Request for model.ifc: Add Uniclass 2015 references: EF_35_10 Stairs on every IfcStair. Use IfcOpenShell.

First a look at what the model holds.

```python
import ifcopenshell

model = ifcopenshell.open("model.ifc")
print(model.schema)
print("classifications:", [c.Name for c in model.by_type("IfcClassification")])
for ifc_class in ("IfcDoor", "IfcRoof", "IfcStair", "IfcWall", "IfcWindow"):
    print(ifc_class, len(model.by_type(ifc_class)))
```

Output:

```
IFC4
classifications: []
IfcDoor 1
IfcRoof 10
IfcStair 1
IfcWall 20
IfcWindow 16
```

```python
import ifcopenshell
import ifcopenshell.api.classification

model = ifcopenshell.open("model.ifc")

system = ifcopenshell.api.classification.add_classification(model, classification="Uniclass 2015")

codes = {
    "IfcStair": ("EF_35_10", "Stairs"),
}
for ifc_class, (code, name) in codes.items():
    products = model.by_type(ifc_class)
    ifcopenshell.api.classification.add_reference(
        model, products=products, classification=system, identification=code, name=name
    )
    print(code, len(products))

model.write("model_edited.ifc")
```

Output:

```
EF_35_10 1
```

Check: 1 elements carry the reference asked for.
